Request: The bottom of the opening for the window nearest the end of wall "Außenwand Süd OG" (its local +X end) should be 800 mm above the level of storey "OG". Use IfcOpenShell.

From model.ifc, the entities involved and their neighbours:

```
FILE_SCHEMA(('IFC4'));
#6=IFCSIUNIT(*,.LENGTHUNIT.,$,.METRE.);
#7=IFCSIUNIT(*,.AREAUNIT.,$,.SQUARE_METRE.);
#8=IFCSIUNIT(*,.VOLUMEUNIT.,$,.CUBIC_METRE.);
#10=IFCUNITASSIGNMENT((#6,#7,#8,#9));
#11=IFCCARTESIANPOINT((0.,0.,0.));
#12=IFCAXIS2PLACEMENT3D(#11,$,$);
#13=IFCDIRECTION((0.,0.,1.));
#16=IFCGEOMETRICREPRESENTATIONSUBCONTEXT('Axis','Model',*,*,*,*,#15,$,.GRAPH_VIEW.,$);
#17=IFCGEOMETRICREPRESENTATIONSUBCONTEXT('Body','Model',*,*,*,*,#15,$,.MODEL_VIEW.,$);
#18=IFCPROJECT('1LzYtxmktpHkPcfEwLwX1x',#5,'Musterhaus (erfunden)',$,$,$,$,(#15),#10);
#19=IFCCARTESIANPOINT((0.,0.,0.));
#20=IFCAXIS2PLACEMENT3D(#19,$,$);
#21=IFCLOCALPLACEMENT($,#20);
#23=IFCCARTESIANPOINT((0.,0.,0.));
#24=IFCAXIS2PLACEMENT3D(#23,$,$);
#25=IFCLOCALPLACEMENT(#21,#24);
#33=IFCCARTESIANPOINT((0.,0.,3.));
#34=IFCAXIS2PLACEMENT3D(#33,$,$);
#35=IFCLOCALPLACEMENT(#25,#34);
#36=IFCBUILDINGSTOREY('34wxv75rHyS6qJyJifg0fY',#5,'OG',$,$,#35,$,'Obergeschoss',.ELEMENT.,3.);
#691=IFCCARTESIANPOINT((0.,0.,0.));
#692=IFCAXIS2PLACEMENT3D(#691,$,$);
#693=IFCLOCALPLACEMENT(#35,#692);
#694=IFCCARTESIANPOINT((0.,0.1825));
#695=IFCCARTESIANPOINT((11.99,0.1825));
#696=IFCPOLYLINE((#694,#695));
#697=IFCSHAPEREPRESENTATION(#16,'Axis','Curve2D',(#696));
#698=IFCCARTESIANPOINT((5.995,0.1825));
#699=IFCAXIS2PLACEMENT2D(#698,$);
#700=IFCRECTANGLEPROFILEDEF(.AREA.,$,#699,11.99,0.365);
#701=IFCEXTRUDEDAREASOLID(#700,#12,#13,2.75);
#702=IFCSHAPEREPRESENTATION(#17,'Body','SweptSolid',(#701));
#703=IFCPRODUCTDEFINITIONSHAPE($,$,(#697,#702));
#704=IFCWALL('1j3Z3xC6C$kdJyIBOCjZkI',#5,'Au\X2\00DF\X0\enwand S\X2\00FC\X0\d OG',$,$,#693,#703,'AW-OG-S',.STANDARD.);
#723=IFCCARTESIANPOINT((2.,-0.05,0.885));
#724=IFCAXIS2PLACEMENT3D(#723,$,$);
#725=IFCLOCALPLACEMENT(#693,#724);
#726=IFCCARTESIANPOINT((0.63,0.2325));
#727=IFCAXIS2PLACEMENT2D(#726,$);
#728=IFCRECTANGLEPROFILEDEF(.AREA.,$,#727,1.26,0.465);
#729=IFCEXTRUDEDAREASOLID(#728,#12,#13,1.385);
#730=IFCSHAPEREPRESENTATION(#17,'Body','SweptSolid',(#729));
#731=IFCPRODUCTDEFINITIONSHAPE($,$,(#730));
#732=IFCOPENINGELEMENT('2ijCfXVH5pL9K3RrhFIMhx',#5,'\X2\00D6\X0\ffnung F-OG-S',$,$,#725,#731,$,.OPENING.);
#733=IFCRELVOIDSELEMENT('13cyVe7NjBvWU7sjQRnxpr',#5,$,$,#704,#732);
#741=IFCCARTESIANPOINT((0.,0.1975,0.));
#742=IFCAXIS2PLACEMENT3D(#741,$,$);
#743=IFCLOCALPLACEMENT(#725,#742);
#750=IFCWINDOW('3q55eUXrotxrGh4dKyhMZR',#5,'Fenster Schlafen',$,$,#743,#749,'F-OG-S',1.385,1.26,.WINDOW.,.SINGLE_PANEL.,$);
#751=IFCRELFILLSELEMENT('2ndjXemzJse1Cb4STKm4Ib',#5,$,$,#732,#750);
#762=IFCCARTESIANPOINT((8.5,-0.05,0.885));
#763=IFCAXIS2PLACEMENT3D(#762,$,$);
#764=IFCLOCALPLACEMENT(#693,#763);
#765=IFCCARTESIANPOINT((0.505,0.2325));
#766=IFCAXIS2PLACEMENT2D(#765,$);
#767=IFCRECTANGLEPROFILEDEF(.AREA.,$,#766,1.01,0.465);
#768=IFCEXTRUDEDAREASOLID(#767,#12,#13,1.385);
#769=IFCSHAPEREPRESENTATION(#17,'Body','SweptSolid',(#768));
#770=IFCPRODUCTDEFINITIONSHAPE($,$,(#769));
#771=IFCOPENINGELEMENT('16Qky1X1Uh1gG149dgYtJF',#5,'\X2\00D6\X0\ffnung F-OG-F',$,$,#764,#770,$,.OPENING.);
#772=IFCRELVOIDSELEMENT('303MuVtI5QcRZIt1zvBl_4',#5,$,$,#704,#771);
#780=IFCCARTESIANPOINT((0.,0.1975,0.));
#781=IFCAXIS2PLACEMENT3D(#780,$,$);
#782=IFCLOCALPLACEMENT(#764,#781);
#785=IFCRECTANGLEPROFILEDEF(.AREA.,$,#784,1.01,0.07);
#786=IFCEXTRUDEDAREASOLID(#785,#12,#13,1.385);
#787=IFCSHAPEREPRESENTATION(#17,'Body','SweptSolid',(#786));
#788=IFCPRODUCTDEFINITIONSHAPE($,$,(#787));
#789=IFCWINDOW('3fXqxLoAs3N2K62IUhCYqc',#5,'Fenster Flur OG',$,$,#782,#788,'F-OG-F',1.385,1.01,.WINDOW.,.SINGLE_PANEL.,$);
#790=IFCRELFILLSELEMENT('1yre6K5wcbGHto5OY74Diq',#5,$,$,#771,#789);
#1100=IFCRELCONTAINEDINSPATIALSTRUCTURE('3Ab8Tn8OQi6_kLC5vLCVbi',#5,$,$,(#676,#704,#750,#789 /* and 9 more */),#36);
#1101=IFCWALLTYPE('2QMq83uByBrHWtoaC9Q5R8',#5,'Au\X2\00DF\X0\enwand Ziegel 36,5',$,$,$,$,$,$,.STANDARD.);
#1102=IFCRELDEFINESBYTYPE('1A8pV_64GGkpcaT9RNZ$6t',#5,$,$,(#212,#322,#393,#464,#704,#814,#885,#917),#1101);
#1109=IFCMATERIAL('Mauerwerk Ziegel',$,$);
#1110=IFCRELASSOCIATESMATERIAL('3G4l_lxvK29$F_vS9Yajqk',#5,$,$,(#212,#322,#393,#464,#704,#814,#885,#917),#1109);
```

```python
import numpy as np
import ifcopenshell
import ifcopenshell.api.geometry
import ifcopenshell.geom
import ifcopenshell.util.element
import ifcopenshell.util.placement
import ifcopenshell.util.shape
import ifcopenshell.util.unit

model = ifcopenshell.open("model.ifc")
unit_scale = ifcopenshell.util.unit.calculate_unit_scale(model)

window = model.by_guid("3fXqxLoAs3N2K62IUhCYqc")
opening = window.FillsVoids[0].RelatingOpeningElement
storey = ifcopenshell.util.element.get_container(window, ifc_class="IfcBuildingStorey")
level = ifcopenshell.util.placement.get_local_placement(storey.ObjectPlacement)[2, 3]

# The opening's origin need not be at the sill, so measure its lowest point.
shape = ifcopenshell.geom.create_shape(ifcopenshell.geom.settings(), opening)
bottom = ifcopenshell.util.shape.get_shape_bottom_elevation(shape, shape.geometry) / unit_scale
dz = level + 0.8 - bottom

shift = np.array([0.0, 0.0, dz])
# The window is placed relative to its opening, so it follows when the opening moves.
matrix = ifcopenshell.util.placement.get_local_placement(opening.ObjectPlacement)
matrix[:3, 3] += shift
ifcopenshell.api.geometry.edit_object_placement(
    model, product=opening, matrix=matrix, is_si=False, should_transform_children=True
)

print(f"moved by {dz * unit_scale:+.3f} m")

model.write("model_v2.ifc")
```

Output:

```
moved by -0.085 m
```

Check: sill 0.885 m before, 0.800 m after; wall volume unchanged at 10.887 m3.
